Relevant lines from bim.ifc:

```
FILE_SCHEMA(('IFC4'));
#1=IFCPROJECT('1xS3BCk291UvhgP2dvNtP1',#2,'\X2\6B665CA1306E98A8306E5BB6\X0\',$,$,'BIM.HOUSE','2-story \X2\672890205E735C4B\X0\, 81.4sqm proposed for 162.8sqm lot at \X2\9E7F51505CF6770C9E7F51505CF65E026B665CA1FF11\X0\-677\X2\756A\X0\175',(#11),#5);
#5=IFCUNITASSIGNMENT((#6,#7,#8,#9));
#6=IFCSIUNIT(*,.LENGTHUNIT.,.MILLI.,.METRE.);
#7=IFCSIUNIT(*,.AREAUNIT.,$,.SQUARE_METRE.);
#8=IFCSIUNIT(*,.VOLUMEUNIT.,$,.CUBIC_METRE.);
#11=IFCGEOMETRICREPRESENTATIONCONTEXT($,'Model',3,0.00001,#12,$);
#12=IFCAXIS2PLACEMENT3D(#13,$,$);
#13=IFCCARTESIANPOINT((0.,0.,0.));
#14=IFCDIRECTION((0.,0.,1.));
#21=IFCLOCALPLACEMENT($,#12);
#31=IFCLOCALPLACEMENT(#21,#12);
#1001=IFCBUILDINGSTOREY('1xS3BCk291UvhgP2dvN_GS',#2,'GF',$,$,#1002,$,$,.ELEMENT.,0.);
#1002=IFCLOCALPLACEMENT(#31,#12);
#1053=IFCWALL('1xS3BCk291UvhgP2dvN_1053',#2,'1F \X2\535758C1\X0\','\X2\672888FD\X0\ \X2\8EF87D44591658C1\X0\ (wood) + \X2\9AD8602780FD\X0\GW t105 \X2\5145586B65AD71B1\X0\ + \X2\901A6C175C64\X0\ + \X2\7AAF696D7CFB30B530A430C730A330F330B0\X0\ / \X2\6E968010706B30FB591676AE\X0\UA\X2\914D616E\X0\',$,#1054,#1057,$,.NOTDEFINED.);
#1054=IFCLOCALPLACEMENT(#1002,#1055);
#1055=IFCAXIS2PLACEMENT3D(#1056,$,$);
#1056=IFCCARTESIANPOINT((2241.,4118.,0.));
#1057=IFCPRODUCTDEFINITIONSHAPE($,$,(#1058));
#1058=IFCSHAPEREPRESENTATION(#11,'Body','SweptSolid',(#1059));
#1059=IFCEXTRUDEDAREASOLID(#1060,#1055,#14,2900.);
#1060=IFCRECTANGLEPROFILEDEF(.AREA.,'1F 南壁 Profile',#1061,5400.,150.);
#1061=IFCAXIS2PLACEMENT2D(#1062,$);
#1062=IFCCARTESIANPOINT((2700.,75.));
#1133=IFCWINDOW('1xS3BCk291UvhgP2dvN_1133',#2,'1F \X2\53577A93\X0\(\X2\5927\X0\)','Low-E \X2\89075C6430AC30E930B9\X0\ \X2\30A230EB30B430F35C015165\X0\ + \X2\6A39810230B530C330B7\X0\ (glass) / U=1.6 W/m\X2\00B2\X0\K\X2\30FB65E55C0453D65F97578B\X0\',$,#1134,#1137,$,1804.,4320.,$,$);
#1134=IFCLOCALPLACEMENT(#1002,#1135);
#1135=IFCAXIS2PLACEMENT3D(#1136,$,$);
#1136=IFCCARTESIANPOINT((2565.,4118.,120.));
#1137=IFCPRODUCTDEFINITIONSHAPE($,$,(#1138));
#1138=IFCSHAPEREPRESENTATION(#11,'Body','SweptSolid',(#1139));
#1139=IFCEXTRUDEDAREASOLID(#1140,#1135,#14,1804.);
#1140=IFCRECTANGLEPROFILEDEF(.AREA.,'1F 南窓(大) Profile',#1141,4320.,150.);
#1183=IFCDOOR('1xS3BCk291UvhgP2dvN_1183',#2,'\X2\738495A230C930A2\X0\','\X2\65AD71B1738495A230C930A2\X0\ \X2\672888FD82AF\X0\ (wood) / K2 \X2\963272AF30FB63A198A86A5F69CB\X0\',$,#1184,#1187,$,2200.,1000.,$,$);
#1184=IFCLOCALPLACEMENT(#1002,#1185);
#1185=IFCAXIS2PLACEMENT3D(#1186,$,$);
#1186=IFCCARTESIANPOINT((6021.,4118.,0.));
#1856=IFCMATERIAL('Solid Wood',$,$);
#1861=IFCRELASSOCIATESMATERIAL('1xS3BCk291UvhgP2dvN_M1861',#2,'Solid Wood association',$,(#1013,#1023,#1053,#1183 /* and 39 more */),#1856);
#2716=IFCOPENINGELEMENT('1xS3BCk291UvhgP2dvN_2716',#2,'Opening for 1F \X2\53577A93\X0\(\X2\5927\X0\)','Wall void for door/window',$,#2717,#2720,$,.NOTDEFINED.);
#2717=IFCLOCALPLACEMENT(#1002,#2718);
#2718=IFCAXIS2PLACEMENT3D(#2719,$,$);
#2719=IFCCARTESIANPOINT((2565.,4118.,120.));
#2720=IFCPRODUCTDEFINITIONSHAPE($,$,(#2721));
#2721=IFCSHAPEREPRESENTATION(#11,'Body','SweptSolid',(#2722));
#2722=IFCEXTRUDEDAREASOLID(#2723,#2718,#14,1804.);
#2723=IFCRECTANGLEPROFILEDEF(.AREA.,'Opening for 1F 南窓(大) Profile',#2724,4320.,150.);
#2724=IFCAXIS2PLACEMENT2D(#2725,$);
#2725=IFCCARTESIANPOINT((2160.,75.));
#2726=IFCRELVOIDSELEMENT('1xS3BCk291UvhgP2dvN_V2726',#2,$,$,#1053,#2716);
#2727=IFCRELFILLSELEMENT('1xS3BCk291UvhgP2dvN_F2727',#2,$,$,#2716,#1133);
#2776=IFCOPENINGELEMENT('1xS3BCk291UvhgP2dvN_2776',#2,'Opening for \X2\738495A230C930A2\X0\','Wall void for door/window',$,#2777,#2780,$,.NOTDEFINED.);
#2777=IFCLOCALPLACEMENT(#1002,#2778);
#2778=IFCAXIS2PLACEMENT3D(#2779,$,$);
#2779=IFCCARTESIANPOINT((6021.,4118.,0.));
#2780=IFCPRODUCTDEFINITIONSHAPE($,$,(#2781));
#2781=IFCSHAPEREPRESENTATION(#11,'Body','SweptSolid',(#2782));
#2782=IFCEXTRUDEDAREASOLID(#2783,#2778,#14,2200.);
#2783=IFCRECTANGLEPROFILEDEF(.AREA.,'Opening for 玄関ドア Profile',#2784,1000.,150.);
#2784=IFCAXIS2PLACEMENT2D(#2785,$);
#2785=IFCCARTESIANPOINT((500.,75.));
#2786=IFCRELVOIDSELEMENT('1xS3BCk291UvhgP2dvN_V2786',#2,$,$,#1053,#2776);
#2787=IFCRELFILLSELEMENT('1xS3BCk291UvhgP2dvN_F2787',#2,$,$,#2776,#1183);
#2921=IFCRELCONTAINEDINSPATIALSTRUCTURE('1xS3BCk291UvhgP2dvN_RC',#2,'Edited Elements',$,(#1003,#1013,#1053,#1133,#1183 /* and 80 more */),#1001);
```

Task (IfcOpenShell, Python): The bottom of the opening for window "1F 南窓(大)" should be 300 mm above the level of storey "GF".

```python
import numpy as np
import ifcopenshell
import ifcopenshell.api.geometry
import ifcopenshell.geom
import ifcopenshell.util.element
import ifcopenshell.util.placement
import ifcopenshell.util.shape
import ifcopenshell.util.unit

model = ifcopenshell.open("bim.ifc")
unit_scale = ifcopenshell.util.unit.calculate_unit_scale(model)

window = model.by_guid("1xS3BCk291UvhgP2dvN_1133")
opening = window.FillsVoids[0].RelatingOpeningElement
storey = ifcopenshell.util.element.get_container(window, ifc_class="IfcBuildingStorey")
level = ifcopenshell.util.placement.get_local_placement(storey.ObjectPlacement)[2, 3]

# The opening's origin need not be at the sill, so measure its lowest point.
shape = ifcopenshell.geom.create_shape(ifcopenshell.geom.settings(), opening)
bottom = ifcopenshell.util.shape.get_shape_bottom_elevation(shape, shape.geometry) / unit_scale
dz = level + 300.0 - bottom

shift = np.array([0.0, 0.0, dz])
# The window is not placed relative to its opening, so move both.
for product in (opening, window):
    matrix = ifcopenshell.util.placement.get_local_placement(product.ObjectPlacement)
    matrix[:3, 3] += shift
    ifcopenshell.api.geometry.edit_object_placement(model, product=product, matrix=matrix, is_si=False)

print(f"moved by {dz * unit_scale:+.3f} m")

model.write("bim_updated.ifc")
```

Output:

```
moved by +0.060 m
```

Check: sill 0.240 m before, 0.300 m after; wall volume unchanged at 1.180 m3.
